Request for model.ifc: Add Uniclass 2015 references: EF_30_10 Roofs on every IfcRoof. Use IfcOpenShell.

First a look at what the model holds.

```python
import ifcopenshell

model = ifcopenshell.open("model.ifc")
print(model.schema)
print("classifications:", [c.Name for c in model.by_type("IfcClassification")])
for ifc_class in ("IfcDoor", "IfcRoof", "IfcStair", "IfcWall", "IfcWindow"):
    print(ifc_class, len(model.by_type(ifc_class)))
```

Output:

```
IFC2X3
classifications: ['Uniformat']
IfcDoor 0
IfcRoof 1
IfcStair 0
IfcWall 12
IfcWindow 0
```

```python
import ifcopenshell
import ifcopenshell.api.classification

model = ifcopenshell.open("model.ifc")

# IFC2X3 requires Source and Edition and has no link from the project to the system.
system = model.create_entity("IfcClassification", Source="NBS", Edition="2015", Name="Uniclass 2015")

codes = {
    "IfcRoof": ("EF_30_10", "Roofs"),
}
for ifc_class, (code, name) in codes.items():
    products = model.by_type(ifc_class)
    ifcopenshell.api.classification.add_reference(
        model, products=products, classification=system, identification=code, name=name
    )
    print(code, len(products))

model.write("model_edited.ifc")
```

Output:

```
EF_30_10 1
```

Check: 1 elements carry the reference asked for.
